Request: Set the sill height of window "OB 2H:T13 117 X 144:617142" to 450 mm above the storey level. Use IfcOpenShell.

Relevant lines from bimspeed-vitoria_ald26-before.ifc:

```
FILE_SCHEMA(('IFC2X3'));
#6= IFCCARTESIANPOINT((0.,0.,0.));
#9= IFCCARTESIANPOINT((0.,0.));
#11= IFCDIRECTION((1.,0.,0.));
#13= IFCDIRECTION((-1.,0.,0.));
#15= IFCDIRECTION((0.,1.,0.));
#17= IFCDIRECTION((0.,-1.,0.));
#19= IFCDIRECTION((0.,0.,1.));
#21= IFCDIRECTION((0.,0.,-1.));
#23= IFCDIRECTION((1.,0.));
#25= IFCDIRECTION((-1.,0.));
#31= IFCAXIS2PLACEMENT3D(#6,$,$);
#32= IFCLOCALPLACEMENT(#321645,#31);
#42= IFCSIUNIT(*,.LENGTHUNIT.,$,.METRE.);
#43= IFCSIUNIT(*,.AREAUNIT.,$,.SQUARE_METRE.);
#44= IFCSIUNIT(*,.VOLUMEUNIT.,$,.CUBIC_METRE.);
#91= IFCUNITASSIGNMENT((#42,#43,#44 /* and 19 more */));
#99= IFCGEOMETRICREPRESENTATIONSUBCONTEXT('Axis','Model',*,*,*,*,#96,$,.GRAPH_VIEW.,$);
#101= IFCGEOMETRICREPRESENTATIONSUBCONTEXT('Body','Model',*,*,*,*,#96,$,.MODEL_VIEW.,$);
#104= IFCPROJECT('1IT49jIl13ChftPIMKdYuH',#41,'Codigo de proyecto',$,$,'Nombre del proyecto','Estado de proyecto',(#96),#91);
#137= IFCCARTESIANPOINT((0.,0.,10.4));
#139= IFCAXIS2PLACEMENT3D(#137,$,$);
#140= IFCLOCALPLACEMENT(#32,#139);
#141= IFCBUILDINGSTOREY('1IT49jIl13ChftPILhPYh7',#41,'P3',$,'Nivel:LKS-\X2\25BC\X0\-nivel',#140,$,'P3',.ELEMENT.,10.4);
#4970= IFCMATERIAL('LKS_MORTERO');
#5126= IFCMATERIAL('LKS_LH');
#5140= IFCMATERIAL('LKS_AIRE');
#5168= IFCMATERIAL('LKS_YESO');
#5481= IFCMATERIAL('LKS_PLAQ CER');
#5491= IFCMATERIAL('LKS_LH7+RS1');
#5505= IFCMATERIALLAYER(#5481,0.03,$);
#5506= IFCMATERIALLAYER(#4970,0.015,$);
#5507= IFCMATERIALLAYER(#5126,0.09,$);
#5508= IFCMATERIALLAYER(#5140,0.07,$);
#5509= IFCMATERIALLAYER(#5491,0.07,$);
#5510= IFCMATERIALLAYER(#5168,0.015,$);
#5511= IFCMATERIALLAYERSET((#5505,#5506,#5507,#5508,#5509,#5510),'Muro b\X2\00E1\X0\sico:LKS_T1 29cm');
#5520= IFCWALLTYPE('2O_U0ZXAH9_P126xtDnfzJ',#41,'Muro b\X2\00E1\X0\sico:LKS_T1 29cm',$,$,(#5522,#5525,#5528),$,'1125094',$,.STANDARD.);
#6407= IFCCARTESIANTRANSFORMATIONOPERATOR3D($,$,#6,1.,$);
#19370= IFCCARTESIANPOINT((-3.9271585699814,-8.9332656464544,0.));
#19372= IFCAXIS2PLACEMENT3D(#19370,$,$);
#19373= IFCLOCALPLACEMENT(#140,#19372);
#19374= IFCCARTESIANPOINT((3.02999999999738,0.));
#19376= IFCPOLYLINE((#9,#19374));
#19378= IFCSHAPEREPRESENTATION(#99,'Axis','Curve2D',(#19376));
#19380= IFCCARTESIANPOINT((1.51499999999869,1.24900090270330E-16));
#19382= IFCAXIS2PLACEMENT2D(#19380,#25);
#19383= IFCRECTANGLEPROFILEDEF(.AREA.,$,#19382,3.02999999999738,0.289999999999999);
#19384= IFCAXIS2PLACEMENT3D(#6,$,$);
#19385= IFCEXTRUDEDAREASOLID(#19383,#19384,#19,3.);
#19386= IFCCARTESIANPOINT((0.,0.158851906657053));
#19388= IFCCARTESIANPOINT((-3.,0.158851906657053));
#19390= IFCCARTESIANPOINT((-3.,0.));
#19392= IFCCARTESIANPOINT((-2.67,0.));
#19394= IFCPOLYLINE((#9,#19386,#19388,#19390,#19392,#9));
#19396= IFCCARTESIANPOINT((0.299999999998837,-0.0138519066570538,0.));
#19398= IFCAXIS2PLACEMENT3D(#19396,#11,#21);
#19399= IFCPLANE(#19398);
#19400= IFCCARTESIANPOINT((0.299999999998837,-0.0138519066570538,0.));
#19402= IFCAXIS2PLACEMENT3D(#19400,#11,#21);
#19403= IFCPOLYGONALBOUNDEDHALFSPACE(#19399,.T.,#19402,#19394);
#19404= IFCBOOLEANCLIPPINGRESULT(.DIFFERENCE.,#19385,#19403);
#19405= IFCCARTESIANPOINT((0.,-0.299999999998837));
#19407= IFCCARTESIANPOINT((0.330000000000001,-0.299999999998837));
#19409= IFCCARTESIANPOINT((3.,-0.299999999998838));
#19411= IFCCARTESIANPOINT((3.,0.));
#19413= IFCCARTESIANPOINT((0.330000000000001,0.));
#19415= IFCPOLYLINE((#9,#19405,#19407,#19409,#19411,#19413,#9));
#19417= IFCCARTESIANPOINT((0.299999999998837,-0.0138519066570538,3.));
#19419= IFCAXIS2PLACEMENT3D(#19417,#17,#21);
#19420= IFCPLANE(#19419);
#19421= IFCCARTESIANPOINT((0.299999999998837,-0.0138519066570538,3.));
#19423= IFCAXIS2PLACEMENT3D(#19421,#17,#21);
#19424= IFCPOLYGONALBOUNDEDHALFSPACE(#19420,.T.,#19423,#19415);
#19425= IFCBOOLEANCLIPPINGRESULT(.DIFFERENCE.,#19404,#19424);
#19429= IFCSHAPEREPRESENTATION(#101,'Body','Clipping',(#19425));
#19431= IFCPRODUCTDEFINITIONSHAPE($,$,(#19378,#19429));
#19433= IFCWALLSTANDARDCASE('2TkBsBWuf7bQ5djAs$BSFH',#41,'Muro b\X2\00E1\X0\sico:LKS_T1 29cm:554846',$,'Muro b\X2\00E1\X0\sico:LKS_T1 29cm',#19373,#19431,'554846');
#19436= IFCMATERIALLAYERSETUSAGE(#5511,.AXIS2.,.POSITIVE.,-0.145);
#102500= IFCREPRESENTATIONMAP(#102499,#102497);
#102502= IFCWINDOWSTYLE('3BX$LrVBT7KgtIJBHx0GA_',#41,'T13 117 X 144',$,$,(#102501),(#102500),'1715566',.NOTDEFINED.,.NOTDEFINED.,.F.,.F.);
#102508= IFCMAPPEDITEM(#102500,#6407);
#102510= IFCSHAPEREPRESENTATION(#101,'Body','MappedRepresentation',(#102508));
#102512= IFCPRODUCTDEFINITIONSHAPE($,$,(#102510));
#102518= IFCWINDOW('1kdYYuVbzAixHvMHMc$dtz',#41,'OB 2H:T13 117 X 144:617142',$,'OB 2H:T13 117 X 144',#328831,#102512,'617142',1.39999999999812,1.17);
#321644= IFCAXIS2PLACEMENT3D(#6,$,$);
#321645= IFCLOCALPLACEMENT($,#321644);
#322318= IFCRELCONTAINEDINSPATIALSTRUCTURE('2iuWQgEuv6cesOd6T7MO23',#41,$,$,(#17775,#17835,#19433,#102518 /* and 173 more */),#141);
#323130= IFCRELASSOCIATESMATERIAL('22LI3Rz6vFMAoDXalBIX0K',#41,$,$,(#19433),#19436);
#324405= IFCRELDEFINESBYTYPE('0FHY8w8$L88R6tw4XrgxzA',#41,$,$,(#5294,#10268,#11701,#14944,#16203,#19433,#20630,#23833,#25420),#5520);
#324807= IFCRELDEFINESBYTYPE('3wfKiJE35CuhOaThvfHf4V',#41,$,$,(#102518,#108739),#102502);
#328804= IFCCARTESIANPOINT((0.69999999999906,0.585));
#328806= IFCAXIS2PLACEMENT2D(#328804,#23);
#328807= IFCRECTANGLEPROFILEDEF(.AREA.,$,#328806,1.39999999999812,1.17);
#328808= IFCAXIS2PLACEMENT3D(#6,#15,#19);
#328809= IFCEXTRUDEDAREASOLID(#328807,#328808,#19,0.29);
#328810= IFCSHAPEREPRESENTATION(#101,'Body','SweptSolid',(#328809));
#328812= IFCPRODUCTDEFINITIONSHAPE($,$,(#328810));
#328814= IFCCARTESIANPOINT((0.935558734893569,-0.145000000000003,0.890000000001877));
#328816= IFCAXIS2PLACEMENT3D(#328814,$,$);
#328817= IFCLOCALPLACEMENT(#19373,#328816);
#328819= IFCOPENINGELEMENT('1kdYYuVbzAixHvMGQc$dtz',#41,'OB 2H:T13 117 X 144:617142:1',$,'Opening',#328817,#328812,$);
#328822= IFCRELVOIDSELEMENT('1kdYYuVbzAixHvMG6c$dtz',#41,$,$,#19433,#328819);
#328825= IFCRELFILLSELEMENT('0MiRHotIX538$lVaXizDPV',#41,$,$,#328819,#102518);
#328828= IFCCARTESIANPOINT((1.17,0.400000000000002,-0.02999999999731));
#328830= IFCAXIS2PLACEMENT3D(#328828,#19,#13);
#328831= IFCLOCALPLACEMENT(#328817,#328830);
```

```python
import numpy as np
import ifcopenshell
import ifcopenshell.api.geometry
import ifcopenshell.geom
import ifcopenshell.util.element
import ifcopenshell.util.placement
import ifcopenshell.util.shape
import ifcopenshell.util.unit

model = ifcopenshell.open("bimspeed-vitoria_ald26-before.ifc")
unit_scale = ifcopenshell.util.unit.calculate_unit_scale(model)

window = model.by_id(102518)
opening = window.FillsVoids[0].RelatingOpeningElement
storey = ifcopenshell.util.element.get_container(window, ifc_class="IfcBuildingStorey")
level = ifcopenshell.util.placement.get_local_placement(storey.ObjectPlacement)[2, 3]

# The opening's origin need not be at the sill, so measure its lowest point.
shape = ifcopenshell.geom.create_shape(ifcopenshell.geom.settings(), opening)
bottom = ifcopenshell.util.shape.get_shape_bottom_elevation(shape, shape.geometry) / unit_scale
dz = level + 0.45 - bottom

shift = np.array([0.0, 0.0, dz])
# The window is placed relative to its opening, so it follows when the opening moves.
matrix = ifcopenshell.util.placement.get_local_placement(opening.ObjectPlacement)
matrix[:3, 3] += shift
ifcopenshell.api.geometry.edit_object_placement(
    model, product=opening, matrix=matrix, is_si=False, should_transform_children=True
)

print(f"moved by {dz * unit_scale:+.3f} m")

model.write("bimspeed-vitoria_ald26-before_updated.ifc")
```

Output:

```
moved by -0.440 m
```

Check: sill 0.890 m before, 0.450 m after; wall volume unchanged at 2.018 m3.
